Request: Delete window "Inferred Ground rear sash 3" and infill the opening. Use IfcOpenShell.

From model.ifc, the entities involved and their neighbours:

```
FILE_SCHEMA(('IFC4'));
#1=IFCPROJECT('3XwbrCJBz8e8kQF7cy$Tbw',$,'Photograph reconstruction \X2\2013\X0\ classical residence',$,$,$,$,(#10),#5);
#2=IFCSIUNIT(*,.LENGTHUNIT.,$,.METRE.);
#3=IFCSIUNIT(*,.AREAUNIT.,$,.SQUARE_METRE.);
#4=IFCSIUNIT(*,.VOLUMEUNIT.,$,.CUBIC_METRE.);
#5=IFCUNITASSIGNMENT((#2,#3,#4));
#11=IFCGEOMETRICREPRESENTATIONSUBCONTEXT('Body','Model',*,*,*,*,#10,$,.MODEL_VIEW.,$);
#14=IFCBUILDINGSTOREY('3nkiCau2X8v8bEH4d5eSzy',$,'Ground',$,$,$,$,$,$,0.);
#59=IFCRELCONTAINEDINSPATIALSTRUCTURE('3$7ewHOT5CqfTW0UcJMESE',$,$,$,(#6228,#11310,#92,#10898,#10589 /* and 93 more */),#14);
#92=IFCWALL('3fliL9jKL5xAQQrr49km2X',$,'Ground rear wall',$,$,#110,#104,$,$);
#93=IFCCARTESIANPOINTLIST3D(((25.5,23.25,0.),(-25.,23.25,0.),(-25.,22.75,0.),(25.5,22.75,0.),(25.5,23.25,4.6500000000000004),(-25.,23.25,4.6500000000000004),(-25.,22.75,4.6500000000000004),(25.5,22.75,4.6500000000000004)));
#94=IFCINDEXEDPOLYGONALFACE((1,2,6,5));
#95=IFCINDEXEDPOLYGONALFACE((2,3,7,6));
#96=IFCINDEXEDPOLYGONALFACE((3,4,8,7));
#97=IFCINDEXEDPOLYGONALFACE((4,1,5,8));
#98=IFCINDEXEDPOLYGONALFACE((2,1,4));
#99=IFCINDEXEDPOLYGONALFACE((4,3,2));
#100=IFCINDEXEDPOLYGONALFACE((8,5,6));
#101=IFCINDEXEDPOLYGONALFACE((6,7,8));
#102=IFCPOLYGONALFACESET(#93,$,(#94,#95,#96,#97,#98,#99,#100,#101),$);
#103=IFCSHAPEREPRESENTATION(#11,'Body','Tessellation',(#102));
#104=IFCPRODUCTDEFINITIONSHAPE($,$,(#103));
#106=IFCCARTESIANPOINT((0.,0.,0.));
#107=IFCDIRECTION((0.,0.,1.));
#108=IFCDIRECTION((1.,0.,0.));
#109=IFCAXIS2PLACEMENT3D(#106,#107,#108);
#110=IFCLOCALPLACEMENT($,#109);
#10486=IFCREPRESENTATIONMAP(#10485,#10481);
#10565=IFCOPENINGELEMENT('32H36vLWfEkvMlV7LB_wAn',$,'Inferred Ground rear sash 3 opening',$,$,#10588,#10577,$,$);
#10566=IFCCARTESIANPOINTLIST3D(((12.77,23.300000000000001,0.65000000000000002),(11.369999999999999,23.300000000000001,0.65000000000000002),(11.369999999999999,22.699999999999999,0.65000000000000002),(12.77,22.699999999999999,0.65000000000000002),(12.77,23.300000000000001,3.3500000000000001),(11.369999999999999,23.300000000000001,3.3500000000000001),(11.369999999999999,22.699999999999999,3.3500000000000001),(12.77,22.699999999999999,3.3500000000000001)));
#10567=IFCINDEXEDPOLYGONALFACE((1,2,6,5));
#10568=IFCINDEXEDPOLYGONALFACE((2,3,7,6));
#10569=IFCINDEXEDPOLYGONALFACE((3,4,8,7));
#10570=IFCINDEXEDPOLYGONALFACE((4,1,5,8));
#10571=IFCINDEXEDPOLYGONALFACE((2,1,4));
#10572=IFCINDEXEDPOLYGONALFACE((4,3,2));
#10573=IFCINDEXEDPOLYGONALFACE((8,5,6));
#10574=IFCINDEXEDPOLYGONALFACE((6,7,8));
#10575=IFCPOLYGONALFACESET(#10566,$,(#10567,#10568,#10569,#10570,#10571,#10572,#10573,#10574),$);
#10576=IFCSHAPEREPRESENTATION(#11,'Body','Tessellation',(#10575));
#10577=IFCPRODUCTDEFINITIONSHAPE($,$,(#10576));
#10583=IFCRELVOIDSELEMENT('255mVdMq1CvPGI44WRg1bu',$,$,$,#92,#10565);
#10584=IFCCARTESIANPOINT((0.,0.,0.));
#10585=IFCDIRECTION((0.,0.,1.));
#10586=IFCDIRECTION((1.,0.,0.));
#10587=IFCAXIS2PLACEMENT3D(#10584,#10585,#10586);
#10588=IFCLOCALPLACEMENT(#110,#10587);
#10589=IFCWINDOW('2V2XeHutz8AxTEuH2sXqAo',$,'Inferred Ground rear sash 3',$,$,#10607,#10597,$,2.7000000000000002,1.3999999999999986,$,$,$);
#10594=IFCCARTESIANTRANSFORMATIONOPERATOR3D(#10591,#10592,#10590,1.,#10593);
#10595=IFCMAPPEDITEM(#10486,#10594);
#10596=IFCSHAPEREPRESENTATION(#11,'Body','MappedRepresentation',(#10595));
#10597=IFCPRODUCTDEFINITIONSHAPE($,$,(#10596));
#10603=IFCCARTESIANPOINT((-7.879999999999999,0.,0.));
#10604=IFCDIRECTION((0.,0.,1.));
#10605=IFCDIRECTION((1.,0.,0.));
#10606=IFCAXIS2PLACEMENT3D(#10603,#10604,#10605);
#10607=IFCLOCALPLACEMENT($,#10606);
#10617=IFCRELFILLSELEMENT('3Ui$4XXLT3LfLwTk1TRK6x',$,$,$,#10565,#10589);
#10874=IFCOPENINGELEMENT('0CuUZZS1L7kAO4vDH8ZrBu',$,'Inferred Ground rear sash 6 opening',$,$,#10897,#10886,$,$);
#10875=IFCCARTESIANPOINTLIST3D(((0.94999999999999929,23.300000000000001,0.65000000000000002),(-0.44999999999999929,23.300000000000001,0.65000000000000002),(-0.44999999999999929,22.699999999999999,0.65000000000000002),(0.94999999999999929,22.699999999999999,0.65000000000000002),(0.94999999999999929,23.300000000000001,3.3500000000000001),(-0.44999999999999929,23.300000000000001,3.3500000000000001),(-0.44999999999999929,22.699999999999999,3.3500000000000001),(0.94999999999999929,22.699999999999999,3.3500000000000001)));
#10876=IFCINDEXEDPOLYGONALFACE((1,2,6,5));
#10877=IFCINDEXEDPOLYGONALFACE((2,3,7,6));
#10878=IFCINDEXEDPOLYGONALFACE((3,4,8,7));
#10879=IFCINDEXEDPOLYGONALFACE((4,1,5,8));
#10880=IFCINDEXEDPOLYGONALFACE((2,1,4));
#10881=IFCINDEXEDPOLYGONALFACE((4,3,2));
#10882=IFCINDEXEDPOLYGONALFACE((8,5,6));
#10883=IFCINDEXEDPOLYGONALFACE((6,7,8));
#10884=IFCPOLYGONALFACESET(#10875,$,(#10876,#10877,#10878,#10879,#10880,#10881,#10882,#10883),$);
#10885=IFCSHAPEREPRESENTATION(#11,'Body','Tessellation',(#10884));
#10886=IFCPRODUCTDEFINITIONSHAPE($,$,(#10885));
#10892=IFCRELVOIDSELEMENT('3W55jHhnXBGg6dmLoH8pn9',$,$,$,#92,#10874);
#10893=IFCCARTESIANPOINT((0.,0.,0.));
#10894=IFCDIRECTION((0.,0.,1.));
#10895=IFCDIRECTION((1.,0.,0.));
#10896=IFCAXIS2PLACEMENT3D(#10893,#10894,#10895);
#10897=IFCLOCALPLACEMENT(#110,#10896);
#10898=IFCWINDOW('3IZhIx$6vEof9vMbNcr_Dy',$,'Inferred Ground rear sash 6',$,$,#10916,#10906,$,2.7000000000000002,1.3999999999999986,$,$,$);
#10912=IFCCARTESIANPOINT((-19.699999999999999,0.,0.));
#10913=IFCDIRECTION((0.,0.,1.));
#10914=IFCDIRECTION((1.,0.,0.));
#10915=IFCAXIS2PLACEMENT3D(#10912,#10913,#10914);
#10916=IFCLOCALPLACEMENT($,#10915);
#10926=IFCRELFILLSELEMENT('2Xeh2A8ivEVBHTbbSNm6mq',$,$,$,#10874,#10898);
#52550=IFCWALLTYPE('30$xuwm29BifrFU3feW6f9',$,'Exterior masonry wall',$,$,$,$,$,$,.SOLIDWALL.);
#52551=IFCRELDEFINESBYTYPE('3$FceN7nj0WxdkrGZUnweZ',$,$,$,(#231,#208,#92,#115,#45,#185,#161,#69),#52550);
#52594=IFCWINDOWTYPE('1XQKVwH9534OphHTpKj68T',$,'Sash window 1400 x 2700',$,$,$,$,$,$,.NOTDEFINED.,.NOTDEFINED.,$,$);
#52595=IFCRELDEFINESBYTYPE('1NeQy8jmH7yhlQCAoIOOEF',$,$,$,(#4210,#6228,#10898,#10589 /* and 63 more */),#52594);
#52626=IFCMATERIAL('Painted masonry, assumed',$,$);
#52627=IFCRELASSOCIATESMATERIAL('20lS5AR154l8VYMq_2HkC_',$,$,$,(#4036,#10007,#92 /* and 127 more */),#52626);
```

```python
import ifcopenshell
import ifcopenshell.api.feature
import ifcopenshell.api.root
import ifcopenshell.geom
import ifcopenshell.util.shape

model = ifcopenshell.open("model.ifc")
settings = ifcopenshell.geom.settings()


def volume(element):
    """Net volume in cubic metres, openings subtracted."""
    shape = ifcopenshell.geom.create_shape(settings, element)
    return ifcopenshell.util.shape.get_volume(shape.geometry)


window = model.by_id(10589)
opening = window.FillsVoids[0].RelatingOpeningElement
wall = opening.VoidsElements[0].RelatingBuildingElement
before = volume(wall)

ifcopenshell.api.root.remove_product(model, product=window)
ifcopenshell.api.feature.remove_feature(model, feature=opening)

after = volume(wall)

print(f"wall volume {before:.3f} -> {after:.3f} m3")

model.write("model-out.ifc")
```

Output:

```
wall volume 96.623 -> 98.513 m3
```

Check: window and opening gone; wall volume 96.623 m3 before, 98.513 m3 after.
